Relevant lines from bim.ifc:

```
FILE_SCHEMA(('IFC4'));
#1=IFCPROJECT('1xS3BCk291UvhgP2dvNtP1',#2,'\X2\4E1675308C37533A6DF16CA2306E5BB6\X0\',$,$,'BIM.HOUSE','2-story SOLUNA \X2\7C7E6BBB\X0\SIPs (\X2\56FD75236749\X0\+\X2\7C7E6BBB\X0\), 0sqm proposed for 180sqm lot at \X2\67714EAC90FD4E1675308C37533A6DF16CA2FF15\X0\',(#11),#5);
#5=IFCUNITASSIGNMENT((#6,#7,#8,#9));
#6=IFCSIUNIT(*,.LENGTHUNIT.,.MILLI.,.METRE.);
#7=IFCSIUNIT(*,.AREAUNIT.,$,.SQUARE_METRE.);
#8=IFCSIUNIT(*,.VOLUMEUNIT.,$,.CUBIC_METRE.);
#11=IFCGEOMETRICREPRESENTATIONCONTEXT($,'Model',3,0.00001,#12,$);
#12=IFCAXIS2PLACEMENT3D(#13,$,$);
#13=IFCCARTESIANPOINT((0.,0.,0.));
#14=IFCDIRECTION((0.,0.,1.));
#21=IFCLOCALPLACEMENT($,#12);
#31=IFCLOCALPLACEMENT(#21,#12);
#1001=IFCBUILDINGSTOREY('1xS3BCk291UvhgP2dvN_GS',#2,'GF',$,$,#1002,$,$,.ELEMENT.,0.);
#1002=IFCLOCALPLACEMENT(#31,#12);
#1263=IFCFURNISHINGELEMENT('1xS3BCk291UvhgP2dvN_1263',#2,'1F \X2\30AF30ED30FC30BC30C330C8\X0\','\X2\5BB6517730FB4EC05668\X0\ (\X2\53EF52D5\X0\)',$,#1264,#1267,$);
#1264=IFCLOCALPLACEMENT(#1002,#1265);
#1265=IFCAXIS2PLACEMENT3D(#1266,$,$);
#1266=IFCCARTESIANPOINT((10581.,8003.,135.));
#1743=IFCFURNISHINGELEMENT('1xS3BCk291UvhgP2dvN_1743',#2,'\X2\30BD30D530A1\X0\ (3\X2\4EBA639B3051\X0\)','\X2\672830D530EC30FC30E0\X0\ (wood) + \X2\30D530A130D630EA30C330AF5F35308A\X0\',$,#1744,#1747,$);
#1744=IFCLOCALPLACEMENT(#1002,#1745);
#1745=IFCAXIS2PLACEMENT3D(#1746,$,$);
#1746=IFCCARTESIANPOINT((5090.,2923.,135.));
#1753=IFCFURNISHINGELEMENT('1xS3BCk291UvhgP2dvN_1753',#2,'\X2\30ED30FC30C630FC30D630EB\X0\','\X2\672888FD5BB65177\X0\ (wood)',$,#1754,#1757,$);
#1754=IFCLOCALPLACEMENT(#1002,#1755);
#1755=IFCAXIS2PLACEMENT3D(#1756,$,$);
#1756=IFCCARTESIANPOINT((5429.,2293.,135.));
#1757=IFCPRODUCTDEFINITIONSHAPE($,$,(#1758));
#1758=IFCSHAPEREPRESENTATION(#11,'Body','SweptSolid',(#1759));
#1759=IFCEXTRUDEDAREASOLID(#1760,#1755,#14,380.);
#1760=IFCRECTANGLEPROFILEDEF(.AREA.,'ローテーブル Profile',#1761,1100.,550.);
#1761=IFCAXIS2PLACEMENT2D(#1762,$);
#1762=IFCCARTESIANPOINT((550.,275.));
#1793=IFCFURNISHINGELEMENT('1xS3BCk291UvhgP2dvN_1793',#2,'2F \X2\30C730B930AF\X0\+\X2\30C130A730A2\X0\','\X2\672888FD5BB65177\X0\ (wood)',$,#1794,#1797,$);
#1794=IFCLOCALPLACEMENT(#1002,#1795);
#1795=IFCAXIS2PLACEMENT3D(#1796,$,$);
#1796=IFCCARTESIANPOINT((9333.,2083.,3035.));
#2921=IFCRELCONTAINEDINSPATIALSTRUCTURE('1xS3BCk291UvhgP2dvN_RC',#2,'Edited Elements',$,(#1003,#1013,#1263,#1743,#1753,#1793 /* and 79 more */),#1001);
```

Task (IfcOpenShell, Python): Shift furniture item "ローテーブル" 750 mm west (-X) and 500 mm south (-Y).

```python
import ifcopenshell
import ifcopenshell.api.geometry
import ifcopenshell.util.placement
import ifcopenshell.util.unit

model = ifcopenshell.open("bim.ifc")
unit_scale = ifcopenshell.util.unit.calculate_unit_scale(model)

item = model.by_guid("1xS3BCk291UvhgP2dvN_1753")
matrix = ifcopenshell.util.placement.get_local_placement(item.ObjectPlacement)
matrix[0, 3] -= 0.75 / unit_scale
matrix[1, 3] -= 0.5 / unit_scale
ifcopenshell.api.geometry.edit_object_placement(model, product=item, matrix=matrix, is_si=False)

print(ifcopenshell.util.placement.get_local_placement(item.ObjectPlacement).round(3) + 0.0)

model.write("bim_rev.ifc")
```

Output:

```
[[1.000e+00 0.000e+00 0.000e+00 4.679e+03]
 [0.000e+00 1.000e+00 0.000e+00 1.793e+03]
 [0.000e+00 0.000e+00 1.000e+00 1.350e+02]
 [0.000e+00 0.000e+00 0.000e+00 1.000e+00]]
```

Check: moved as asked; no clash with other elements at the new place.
